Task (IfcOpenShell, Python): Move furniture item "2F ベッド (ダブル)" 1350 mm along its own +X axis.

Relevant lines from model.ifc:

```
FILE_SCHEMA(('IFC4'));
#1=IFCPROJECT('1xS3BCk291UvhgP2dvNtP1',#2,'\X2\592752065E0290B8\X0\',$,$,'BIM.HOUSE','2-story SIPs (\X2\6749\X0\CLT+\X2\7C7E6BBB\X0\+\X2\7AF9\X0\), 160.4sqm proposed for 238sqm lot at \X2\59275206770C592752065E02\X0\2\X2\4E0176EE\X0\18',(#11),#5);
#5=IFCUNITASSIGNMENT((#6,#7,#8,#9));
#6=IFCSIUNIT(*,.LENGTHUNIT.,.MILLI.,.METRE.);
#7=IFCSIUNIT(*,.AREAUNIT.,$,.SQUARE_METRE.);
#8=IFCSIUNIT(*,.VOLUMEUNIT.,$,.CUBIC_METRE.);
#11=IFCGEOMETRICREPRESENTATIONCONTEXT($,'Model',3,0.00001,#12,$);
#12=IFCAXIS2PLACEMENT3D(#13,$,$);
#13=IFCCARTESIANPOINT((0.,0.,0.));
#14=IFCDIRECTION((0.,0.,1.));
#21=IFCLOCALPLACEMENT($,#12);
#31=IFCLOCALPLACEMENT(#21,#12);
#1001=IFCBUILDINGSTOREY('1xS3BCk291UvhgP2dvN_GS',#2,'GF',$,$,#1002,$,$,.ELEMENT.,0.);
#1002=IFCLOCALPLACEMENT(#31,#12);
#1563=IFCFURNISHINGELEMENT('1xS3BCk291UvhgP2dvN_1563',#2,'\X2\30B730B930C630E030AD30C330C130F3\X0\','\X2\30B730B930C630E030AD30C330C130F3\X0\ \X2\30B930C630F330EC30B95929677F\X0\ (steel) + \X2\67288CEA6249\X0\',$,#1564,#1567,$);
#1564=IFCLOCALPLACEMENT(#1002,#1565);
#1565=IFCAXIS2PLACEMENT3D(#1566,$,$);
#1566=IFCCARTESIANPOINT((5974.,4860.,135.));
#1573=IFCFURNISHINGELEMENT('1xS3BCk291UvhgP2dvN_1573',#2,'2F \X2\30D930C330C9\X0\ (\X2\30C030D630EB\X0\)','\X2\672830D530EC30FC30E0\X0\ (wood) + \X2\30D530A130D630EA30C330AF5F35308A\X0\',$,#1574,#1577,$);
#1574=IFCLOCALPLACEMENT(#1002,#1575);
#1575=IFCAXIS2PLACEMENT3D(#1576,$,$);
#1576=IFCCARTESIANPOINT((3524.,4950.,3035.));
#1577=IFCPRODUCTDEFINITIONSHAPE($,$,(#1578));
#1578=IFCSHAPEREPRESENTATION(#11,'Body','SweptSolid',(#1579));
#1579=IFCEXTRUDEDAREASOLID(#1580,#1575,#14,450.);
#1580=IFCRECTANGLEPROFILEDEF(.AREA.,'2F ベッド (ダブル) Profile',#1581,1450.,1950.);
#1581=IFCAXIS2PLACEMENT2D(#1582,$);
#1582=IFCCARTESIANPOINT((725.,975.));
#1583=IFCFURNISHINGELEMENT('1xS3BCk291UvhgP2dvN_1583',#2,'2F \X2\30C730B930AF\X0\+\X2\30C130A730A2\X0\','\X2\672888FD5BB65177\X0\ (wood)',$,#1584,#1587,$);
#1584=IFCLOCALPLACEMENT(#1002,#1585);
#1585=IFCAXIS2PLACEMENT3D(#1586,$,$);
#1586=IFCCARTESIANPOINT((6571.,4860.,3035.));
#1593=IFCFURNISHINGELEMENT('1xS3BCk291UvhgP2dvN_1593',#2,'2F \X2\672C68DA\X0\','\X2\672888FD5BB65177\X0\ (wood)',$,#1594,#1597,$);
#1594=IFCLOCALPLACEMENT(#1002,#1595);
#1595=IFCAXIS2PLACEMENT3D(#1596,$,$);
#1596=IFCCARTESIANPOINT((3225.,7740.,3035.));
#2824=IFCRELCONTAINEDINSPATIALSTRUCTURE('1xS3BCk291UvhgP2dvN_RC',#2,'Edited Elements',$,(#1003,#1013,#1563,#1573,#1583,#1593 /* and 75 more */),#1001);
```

```python
import ifcopenshell
import ifcopenshell.api.geometry
import ifcopenshell.util.placement

model = ifcopenshell.open("model.ifc")

item = model.by_guid("1xS3BCk291UvhgP2dvN_1573")
matrix = ifcopenshell.util.placement.get_local_placement(item.ObjectPlacement)
matrix[:3, 3] += matrix[:3, 0] * 1350.0
ifcopenshell.api.geometry.edit_object_placement(model, product=item, matrix=matrix, is_si=False)

print(ifcopenshell.util.placement.get_local_placement(item.ObjectPlacement).round(3) + 0.0)

model.write("model_v2.ifc")
```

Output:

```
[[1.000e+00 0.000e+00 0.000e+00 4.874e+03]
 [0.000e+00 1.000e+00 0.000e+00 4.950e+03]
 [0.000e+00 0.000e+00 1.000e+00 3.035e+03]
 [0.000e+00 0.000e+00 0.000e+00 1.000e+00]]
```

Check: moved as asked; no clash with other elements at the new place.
